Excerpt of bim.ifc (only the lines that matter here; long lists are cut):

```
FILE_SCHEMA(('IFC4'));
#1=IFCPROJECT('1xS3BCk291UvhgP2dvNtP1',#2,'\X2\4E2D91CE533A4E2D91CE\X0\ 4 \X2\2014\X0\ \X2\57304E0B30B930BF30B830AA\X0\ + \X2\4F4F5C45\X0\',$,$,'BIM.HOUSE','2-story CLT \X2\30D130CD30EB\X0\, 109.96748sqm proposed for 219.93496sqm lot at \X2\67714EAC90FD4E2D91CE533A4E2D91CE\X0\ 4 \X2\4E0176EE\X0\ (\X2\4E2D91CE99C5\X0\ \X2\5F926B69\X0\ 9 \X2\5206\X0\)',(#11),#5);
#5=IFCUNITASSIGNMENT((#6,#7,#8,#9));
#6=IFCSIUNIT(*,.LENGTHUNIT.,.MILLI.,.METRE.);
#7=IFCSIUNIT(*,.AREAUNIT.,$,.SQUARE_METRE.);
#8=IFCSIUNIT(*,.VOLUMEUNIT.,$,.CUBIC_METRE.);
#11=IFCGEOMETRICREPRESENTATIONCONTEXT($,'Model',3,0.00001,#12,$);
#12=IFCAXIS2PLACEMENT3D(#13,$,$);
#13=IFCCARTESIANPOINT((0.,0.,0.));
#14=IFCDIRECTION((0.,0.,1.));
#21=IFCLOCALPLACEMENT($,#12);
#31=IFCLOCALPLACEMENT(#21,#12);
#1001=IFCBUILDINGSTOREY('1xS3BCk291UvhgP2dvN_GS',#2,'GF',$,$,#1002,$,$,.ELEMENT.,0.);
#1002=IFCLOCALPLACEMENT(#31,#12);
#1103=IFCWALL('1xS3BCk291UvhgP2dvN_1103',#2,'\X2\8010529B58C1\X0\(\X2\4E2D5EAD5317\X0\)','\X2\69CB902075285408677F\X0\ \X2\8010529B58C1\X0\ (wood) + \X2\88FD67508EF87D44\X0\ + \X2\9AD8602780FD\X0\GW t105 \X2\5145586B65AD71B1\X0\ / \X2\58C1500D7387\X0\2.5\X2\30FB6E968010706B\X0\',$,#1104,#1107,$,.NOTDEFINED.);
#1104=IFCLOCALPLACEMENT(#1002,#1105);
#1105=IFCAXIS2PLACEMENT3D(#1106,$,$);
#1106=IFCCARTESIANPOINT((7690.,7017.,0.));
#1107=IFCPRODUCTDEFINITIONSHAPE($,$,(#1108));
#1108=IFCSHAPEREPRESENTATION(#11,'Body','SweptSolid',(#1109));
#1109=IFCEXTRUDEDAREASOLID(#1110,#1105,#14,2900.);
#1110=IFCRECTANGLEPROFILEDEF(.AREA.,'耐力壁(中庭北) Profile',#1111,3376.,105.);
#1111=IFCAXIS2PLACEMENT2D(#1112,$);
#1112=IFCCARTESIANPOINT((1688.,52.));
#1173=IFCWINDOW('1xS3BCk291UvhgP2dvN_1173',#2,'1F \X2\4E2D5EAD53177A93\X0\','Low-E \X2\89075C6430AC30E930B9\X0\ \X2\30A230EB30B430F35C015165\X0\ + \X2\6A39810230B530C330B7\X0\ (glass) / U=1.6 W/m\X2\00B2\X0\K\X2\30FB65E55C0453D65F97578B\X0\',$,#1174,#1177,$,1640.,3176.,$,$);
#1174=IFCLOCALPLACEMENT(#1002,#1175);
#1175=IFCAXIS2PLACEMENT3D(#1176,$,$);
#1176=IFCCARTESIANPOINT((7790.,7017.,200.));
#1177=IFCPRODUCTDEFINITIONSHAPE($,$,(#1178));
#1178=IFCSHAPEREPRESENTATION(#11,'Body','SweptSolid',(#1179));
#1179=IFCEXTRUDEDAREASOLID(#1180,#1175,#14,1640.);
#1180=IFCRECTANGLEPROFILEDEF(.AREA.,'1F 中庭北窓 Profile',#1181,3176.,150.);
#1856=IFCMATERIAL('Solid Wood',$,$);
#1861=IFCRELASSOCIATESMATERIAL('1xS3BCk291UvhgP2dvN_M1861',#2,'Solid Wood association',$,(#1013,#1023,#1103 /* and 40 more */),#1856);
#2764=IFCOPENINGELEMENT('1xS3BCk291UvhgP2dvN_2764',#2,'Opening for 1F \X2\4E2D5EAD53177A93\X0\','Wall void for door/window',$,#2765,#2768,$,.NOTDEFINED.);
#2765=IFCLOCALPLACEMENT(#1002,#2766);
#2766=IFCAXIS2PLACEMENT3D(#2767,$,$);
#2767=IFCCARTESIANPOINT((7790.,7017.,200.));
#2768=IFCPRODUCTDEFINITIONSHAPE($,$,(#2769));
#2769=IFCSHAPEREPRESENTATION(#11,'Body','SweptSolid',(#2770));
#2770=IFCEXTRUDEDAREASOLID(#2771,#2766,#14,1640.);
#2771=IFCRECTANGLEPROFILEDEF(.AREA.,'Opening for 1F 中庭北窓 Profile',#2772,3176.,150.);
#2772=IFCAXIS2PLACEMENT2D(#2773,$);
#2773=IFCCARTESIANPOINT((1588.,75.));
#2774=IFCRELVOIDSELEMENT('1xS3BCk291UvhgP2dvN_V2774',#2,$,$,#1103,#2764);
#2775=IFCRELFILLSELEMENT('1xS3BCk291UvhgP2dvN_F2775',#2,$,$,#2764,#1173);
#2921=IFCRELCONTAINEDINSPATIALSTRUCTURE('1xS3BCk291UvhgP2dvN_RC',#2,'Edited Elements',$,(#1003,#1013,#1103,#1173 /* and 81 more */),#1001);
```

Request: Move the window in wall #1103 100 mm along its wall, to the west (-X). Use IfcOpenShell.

```python
import ifcopenshell
import ifcopenshell.api.geometry
import ifcopenshell.util.placement
import ifcopenshell.util.unit

model = ifcopenshell.open("bim.ifc")
unit_scale = ifcopenshell.util.unit.calculate_unit_scale(model)

window = model.by_guid("1xS3BCk291UvhgP2dvN_1173")
opening = window.FillsVoids[0].RelatingOpeningElement
wall = opening.VoidsElements[0].RelatingBuildingElement

wall_matrix = ifcopenshell.util.placement.get_local_placement(wall.ObjectPlacement)
shift = wall_matrix[:3, 0] * -0.1 / unit_scale
before = ifcopenshell.util.placement.get_local_placement(window.ObjectPlacement)[:3, 3].copy()

# The window is not placed relative to its opening, so move both.
for product in (opening, window):
    matrix = ifcopenshell.util.placement.get_local_placement(product.ObjectPlacement)
    matrix[:3, 3] += shift
    ifcopenshell.api.geometry.edit_object_placement(model, product=product, matrix=matrix, is_si=False)

after = ifcopenshell.util.placement.get_local_placement(window.ObjectPlacement)[:3, 3]
print("window moved by", (after - before).round(3) + 0.0)

model.write("bim_v2.ifc")
```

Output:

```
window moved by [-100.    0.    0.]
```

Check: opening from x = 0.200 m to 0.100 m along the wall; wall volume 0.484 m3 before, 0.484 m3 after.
